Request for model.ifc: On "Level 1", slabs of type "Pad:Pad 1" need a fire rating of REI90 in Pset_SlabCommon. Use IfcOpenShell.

First a look at what the model holds.

```python
import ifcopenshell
import ifcopenshell.util.element

model = ifcopenshell.open("model.ifc")
print(model.schema)
storey = next(s for s in model.by_type("IfcBuildingStorey") if s.Name == "Level 1")
slabs = [e for e in ifcopenshell.util.element.get_decomposition(storey) if e.is_a("IfcSlab")]
seen = {}
for e in slabs:
    element_type = ifcopenshell.util.element.get_type(e)
    key = (element_type.Name if element_type != e and element_type else None, ifcopenshell.util.element.get_pset(e, "Pset_SlabCommon", "FireRating"))
    seen[key] = seen.get(key, 0) + 1
for (name, value), count in sorted(seen.items(), key=str):
    print(count, "x", name, "|", value)
```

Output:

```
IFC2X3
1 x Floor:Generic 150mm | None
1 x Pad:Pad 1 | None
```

```python
import ifcopenshell
import ifcopenshell.api.pset
import ifcopenshell.util.element

model = ifcopenshell.open("model.ifc")

storey = next(s for s in model.by_type("IfcBuildingStorey") if s.Name == "Level 1")
slabs = [e for e in ifcopenshell.util.element.get_decomposition(storey) if e.is_a("IfcSlab")]

count = 0
for e in slabs:
    element_type = ifcopenshell.util.element.get_type(e)
    if element_type in (None, e) or element_type.Name != "Pad:Pad 1":
        continue
    # add_pset returns the element's existing set when there is one.
    pset = ifcopenshell.api.pset.add_pset(model, product=e, name="Pset_SlabCommon")
    ifcopenshell.api.pset.edit_pset(model, pset=pset, properties={"FireRating": "REI90"})
    count += 1

print(count, "slabs updated")

model.write("model_edited.ifc")
```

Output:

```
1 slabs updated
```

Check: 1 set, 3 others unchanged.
